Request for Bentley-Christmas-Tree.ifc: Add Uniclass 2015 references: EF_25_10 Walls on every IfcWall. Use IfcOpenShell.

First a look at what the model holds.

```python
import ifcopenshell

model = ifcopenshell.open("Bentley-Christmas-Tree.ifc")
print(model.schema)
print("classifications:", [c.Name for c in model.by_type("IfcClassification")])
for ifc_class in ("IfcDoor", "IfcRoof", "IfcStair", "IfcWall", "IfcWindow"):
    print(ifc_class, len(model.by_type(ifc_class)))
```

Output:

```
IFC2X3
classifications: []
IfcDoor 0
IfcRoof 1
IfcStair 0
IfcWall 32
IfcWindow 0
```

```python
import ifcopenshell
import ifcopenshell.api.classification

model = ifcopenshell.open("Bentley-Christmas-Tree.ifc")

# IFC2X3 requires Source and Edition and has no link from the project to the system.
system = model.create_entity("IfcClassification", Source="NBS", Edition="2015", Name="Uniclass 2015")

codes = {
    "IfcWall": ("EF_25_10", "Walls"),
}
for ifc_class, (code, name) in codes.items():
    products = model.by_type(ifc_class)
    ifcopenshell.api.classification.add_reference(
        model, products=products, classification=system, identification=code, name=name
    )
    print(code, len(products))

model.write("Bentley-Christmas-Tree_updated.ifc")
```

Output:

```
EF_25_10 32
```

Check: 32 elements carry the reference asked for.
